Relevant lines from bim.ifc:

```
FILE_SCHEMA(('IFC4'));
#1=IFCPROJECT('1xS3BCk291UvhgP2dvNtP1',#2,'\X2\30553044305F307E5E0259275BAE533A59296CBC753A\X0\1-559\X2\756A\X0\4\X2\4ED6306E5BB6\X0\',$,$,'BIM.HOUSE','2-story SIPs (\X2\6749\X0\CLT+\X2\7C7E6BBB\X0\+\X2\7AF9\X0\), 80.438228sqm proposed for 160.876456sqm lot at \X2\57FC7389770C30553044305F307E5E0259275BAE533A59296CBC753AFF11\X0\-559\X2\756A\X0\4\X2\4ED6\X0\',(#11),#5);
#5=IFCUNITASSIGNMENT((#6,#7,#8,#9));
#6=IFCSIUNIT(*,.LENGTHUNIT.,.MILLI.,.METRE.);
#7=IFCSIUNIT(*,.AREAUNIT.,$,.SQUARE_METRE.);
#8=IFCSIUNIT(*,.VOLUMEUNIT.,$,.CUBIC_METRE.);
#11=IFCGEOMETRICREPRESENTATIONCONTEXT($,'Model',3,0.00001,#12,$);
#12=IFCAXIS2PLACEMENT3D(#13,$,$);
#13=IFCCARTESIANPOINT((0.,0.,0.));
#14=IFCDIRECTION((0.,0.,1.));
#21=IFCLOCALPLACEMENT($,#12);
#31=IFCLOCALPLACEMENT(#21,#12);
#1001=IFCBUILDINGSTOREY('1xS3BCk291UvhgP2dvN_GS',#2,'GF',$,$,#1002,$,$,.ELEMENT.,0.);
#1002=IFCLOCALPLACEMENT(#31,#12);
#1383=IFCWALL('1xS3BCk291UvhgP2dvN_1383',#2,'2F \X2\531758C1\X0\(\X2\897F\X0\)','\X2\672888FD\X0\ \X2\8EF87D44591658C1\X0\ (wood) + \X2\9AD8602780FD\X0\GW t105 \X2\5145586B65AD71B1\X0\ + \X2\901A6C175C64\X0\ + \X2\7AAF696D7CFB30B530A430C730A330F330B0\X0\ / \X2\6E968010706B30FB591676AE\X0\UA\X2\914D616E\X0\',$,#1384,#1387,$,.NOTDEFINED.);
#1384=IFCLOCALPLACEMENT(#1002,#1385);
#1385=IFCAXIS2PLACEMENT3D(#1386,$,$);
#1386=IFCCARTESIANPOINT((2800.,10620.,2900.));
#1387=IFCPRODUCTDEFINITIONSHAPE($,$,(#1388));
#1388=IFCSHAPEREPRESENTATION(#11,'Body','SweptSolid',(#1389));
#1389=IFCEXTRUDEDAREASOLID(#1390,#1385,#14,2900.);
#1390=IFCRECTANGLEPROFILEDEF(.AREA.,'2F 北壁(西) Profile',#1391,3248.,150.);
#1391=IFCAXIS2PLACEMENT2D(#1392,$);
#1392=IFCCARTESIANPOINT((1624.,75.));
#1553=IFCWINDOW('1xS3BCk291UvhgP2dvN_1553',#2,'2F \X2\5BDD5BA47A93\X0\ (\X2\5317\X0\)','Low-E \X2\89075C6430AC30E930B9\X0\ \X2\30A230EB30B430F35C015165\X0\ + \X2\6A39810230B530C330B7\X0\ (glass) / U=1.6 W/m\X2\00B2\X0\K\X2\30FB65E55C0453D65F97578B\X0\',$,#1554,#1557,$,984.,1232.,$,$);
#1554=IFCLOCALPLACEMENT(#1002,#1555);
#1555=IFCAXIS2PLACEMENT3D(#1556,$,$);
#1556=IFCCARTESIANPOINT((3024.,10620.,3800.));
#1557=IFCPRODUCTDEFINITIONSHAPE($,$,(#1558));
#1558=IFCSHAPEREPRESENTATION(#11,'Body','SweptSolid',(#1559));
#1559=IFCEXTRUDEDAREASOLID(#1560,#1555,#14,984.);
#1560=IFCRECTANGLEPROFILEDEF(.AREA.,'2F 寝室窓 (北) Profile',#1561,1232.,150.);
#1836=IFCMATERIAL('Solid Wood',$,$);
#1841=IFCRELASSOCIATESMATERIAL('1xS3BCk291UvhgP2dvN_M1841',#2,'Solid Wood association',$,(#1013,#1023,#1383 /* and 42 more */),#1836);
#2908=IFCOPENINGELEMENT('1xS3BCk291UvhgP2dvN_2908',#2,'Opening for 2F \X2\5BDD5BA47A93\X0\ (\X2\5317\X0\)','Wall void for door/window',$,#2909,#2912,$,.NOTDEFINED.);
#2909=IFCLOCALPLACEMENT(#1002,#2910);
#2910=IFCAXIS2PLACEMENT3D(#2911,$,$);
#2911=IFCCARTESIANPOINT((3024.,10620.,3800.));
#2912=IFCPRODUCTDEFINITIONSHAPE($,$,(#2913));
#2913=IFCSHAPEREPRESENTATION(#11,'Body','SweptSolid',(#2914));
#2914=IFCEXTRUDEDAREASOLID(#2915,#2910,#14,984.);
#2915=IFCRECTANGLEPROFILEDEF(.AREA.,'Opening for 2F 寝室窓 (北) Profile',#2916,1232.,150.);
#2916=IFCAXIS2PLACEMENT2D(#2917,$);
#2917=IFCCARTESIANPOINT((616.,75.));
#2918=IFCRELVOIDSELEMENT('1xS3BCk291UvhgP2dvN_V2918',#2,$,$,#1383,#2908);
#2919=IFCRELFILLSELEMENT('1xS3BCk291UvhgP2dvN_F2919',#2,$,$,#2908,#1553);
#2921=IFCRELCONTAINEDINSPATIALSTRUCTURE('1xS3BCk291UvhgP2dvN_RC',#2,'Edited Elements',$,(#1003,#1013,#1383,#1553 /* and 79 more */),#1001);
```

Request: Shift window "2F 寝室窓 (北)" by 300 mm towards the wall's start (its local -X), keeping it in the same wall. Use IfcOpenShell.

```python
import ifcopenshell
import ifcopenshell.api.geometry
import ifcopenshell.util.placement
import ifcopenshell.util.unit

model = ifcopenshell.open("bim.ifc")
unit_scale = ifcopenshell.util.unit.calculate_unit_scale(model)

window = model.by_id(1553)
opening = window.FillsVoids[0].RelatingOpeningElement
wall = opening.VoidsElements[0].RelatingBuildingElement

wall_matrix = ifcopenshell.util.placement.get_local_placement(wall.ObjectPlacement)
shift = wall_matrix[:3, 0] * -0.3 / unit_scale
before = ifcopenshell.util.placement.get_local_placement(window.ObjectPlacement)[:3, 3].copy()

# The window is not placed relative to its opening, so move both.
for product in (opening, window):
    matrix = ifcopenshell.util.placement.get_local_placement(product.ObjectPlacement)
    matrix[:3, 3] += shift
    ifcopenshell.api.geometry.edit_object_placement(model, product=product, matrix=matrix, is_si=False)

after = ifcopenshell.util.placement.get_local_placement(window.ObjectPlacement)[:3, 3]
print("window moved by", (after - before).round(3) + 0.0)

model.write("bim-out.ifc")
```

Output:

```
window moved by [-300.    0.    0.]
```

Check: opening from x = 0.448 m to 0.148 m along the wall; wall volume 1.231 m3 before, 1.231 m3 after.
